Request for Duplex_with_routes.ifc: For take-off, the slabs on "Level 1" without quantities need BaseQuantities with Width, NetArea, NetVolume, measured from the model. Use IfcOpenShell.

First a look at what the model holds.

```python
import ifcopenshell
import ifcopenshell.util.element
import ifcopenshell.util.unit

model = ifcopenshell.open("Duplex_with_routes.ifc")
print(model.schema)
for unit_type in ("LENGTHUNIT", "AREAUNIT", "VOLUMEUNIT"):
    print(unit_type, ifcopenshell.util.unit.calculate_unit_scale(model, unit_type))
storey = next(s for s in model.by_type("IfcBuildingStorey") if s.Name == "Level 1")
slabs = [e for e in ifcopenshell.util.element.get_decomposition(storey) if e.is_a("IfcSlab")]
for e in sorted(slabs, key=lambda e: e.id()):
    print(e.id(), e.is_a(), e.Name, list(ifcopenshell.util.element.get_psets(e, qtos_only=True)), sep=" | ")
```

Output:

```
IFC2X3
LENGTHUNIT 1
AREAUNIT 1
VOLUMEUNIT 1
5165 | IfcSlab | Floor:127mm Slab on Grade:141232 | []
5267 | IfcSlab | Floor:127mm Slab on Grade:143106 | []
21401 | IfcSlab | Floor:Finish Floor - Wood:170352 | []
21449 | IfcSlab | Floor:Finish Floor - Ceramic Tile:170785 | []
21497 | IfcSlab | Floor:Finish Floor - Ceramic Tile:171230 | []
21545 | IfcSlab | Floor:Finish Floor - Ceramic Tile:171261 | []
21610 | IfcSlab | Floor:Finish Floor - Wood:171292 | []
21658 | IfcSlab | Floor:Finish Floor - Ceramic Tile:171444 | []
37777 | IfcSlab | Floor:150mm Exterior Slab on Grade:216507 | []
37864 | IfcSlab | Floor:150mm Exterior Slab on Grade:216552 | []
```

```python
import ifcopenshell
import ifcopenshell.api.pset
import ifcopenshell.geom
import ifcopenshell.util.element
import ifcopenshell.util.shape
import ifcopenshell.util.unit

model = ifcopenshell.open("Duplex_with_routes.ifc")
unit_scale = ifcopenshell.util.unit.calculate_unit_scale(model)
area_scale = ifcopenshell.util.unit.calculate_unit_scale(model, "AREAUNIT")
volume_scale = ifcopenshell.util.unit.calculate_unit_scale(model, "VOLUMEUNIT")
settings = ifcopenshell.geom.settings()

storey = next(s for s in model.by_type("IfcBuildingStorey") if s.Name == "Level 1")
slabs = [e for e in ifcopenshell.util.element.get_decomposition(storey) if e.is_a("IfcSlab")]

for e in sorted(slabs, key=lambda e: e.id()):
    if ifcopenshell.util.element.get_psets(e, qtos_only=True, should_inherit=False):
        continue
    # Geometry comes back in metres, in the element's own axes.
    shape = ifcopenshell.geom.create_shape(settings, e)
    values = {
        "Width": ifcopenshell.util.shape.get_z(shape.geometry) / unit_scale,
        "NetArea": ifcopenshell.util.shape.get_footprint_area(shape.geometry) / area_scale,
        "NetVolume": ifcopenshell.util.shape.get_volume(shape.geometry) / volume_scale,
    }
    qto = ifcopenshell.api.pset.add_qto(model, product=e, name="BaseQuantities")
    ifcopenshell.api.pset.edit_qto(model, qto=qto, properties=values)
    print(e.id(), {k: round(v, 3) for k, v in values.items()})

model.write("Duplex_with_routes_rev.ifc")
```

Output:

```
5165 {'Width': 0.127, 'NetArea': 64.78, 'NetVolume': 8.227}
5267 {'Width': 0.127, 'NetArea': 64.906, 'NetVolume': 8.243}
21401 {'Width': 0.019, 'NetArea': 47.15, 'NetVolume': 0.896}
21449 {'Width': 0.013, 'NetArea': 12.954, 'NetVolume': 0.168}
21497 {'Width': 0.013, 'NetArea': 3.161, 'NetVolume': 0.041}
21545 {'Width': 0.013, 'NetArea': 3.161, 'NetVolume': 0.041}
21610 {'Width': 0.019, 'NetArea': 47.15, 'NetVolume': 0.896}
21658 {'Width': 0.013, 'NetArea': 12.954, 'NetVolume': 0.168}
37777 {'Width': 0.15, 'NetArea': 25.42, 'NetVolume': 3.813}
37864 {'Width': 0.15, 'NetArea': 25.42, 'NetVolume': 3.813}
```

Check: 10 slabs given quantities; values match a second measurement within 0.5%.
